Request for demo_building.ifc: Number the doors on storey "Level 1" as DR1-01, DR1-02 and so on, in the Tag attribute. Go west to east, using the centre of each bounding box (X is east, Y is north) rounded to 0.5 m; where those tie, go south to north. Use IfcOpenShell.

First a look at what the model holds.

```python
import ifcopenshell
import ifcopenshell.util.element
import ifcopenshell.util.placement

model = ifcopenshell.open("demo_building.ifc")
print(model.schema)
storey = next(s for s in model.by_type("IfcBuildingStorey") if s.Name == "Level 1")
doors = [e for e in ifcopenshell.util.element.get_decomposition(storey) if e.is_a("IfcDoor")]
for e in sorted(doors, key=lambda e: e.id()):
    origin = ifcopenshell.util.placement.get_local_placement(e.ObjectPlacement)[:3, 3]
    print(e.id(), e.Tag, e.Name, origin.round(2) + 0.0, sep=" | ")
```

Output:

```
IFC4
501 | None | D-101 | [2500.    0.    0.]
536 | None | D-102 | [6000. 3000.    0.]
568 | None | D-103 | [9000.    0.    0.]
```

```python
import ifcopenshell
import ifcopenshell.geom
import ifcopenshell.util.element
import ifcopenshell.util.shape

model = ifcopenshell.open("demo_building.ifc")
settings = ifcopenshell.geom.settings()
settings.set("use-world-coords", True)


def centre(element):
    shape = ifcopenshell.geom.create_shape(settings, element)
    return ifcopenshell.util.shape.get_bbox_centroid(shape.geometry)


storey = next(s for s in model.by_type("IfcBuildingStorey") if s.Name == "Level 1")
doors = [e for e in ifcopenshell.util.element.get_decomposition(storey) if e.is_a("IfcDoor")]

# Insertion points can sit at a corner or the storey origin, so sort by the geometry (in metres).
centres = {e: centre(e) for e in doors}
doors.sort(key=lambda e: (round(centres[e][0] / 0.5), centres[e][1]))

for i, e in enumerate(doors, start=1):
    number = f"DR1-{i:02d}"
    e.Tag = number
    print(e.id(), number)

model.write("demo_building_v2.ifc")
```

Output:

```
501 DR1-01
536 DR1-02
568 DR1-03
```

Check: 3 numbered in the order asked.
